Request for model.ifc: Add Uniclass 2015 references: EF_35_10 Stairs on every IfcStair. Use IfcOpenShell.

First a look at what the model holds.

```python
import ifcopenshell

model = ifcopenshell.open("model.ifc")
print(model.schema)
print("classifications:", [c.Name for c in model.by_type("IfcClassification")])
for ifc_class in ("IfcDoor", "IfcRoof", "IfcStair", "IfcWall", "IfcWindow"):
    print(ifc_class, len(model.by_type(ifc_class)))
```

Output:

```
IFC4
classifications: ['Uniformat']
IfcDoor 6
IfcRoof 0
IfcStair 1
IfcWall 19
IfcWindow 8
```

```python
import ifcopenshell
import ifcopenshell.api.classification

model = ifcopenshell.open("model.ifc")

system = ifcopenshell.api.classification.add_classification(model, classification="Uniclass 2015")

codes = {
    "IfcStair": ("EF_35_10", "Stairs"),
}
for ifc_class, (code, name) in codes.items():
    products = model.by_type(ifc_class)
    ifcopenshell.api.classification.add_reference(
        model, products=products, classification=system, identification=code, name=name
    )
    print(code, len(products))

model.write("model_rev.ifc")
```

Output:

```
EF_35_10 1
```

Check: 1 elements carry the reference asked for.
